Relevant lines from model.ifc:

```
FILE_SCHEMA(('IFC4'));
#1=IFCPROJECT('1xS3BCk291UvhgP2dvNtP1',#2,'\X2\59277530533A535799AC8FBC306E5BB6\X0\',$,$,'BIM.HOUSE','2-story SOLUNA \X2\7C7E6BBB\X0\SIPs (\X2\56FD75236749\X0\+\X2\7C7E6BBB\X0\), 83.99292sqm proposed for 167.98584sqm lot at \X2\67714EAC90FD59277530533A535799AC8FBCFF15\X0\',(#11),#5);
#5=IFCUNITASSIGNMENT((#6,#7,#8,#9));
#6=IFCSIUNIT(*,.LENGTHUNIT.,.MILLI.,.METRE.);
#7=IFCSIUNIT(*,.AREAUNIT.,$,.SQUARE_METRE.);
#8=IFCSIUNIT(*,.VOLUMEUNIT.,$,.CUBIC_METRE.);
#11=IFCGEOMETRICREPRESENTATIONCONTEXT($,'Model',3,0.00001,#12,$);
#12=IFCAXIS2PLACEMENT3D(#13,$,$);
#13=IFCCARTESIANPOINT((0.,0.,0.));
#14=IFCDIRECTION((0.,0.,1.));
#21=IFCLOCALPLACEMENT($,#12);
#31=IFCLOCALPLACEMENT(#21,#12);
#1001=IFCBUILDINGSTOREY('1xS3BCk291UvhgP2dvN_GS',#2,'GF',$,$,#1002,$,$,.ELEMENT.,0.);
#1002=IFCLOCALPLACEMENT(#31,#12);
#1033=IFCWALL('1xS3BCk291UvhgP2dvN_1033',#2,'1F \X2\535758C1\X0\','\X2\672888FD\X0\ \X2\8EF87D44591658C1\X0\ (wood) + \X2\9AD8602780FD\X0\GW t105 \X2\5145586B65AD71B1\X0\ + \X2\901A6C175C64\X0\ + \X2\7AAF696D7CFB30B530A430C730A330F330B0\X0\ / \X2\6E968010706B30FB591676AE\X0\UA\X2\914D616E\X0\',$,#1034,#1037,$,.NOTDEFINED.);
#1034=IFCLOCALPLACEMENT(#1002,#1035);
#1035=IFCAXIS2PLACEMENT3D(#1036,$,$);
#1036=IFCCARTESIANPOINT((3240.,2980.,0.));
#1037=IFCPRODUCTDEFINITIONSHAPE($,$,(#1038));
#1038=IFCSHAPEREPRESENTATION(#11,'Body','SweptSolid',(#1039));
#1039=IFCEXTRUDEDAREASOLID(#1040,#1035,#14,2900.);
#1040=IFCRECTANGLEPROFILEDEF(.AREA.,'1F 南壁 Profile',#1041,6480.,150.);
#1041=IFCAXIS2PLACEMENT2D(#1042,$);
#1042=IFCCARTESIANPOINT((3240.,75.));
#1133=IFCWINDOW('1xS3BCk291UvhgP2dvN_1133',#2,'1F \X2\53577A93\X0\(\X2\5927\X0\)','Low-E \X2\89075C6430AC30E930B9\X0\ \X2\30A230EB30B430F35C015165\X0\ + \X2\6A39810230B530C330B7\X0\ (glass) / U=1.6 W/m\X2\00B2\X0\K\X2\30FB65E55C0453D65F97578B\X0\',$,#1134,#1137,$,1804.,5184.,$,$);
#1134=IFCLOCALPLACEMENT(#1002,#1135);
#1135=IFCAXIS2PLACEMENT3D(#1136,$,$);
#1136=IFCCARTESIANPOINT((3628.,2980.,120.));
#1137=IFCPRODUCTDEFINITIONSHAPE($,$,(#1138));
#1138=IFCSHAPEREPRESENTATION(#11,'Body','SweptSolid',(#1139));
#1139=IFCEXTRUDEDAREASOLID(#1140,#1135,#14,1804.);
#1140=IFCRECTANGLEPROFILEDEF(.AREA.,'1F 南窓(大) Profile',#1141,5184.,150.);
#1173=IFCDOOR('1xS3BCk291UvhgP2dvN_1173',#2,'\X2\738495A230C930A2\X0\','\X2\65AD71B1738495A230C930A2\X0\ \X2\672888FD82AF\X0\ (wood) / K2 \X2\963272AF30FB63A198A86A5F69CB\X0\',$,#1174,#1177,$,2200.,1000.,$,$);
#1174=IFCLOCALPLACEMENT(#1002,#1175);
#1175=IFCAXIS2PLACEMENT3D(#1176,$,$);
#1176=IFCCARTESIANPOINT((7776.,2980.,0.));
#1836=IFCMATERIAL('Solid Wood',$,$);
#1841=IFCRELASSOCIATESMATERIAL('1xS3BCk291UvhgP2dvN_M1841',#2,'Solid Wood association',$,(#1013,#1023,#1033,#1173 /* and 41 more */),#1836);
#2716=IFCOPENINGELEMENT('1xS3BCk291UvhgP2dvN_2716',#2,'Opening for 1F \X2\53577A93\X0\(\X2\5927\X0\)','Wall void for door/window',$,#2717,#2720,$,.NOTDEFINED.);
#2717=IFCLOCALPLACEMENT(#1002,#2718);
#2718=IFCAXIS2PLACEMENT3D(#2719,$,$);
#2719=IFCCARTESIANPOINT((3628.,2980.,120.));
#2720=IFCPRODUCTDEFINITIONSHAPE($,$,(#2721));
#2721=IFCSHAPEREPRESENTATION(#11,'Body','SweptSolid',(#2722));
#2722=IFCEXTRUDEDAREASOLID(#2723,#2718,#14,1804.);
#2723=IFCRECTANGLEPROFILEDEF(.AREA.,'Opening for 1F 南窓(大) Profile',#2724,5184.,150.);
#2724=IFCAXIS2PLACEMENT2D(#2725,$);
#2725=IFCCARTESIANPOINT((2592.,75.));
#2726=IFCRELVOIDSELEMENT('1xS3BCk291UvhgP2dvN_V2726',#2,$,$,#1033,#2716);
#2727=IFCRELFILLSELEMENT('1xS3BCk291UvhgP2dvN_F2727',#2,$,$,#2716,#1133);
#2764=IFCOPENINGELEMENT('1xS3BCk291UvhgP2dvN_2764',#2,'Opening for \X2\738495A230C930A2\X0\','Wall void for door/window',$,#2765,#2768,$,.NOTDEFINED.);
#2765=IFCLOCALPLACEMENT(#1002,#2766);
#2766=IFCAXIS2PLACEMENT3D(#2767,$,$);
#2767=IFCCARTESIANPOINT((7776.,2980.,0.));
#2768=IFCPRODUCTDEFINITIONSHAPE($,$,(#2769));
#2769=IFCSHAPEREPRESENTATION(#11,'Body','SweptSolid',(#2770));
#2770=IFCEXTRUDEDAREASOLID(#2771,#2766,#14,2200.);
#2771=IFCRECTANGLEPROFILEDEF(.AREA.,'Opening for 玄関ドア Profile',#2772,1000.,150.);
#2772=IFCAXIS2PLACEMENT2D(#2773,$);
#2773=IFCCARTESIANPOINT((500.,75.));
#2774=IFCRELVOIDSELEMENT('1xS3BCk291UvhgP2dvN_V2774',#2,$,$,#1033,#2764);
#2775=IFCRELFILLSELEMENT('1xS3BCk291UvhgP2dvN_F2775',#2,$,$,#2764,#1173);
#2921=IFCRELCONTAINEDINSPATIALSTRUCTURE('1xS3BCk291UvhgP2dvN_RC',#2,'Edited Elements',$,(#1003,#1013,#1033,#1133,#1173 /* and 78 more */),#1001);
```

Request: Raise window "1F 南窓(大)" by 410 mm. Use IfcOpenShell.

```python
import numpy as np
import ifcopenshell
import ifcopenshell.api.geometry
import ifcopenshell.util.placement
import ifcopenshell.util.unit

model = ifcopenshell.open("model.ifc")
unit_scale = ifcopenshell.util.unit.calculate_unit_scale(model)

window = model.by_guid("1xS3BCk291UvhgP2dvN_1133")
opening = window.FillsVoids[0].RelatingOpeningElement
dz = 0.41 / unit_scale

shift = np.array([0.0, 0.0, dz])
# The window is not placed relative to its opening, so move both.
for product in (opening, window):
    matrix = ifcopenshell.util.placement.get_local_placement(product.ObjectPlacement)
    matrix[:3, 3] += shift
    ifcopenshell.api.geometry.edit_object_placement(model, product=product, matrix=matrix, is_si=False)

print(f"moved by {dz * unit_scale:+.3f} m")

model.write("model_v2.ifc")
```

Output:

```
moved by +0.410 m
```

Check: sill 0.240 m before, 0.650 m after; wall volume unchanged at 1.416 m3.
